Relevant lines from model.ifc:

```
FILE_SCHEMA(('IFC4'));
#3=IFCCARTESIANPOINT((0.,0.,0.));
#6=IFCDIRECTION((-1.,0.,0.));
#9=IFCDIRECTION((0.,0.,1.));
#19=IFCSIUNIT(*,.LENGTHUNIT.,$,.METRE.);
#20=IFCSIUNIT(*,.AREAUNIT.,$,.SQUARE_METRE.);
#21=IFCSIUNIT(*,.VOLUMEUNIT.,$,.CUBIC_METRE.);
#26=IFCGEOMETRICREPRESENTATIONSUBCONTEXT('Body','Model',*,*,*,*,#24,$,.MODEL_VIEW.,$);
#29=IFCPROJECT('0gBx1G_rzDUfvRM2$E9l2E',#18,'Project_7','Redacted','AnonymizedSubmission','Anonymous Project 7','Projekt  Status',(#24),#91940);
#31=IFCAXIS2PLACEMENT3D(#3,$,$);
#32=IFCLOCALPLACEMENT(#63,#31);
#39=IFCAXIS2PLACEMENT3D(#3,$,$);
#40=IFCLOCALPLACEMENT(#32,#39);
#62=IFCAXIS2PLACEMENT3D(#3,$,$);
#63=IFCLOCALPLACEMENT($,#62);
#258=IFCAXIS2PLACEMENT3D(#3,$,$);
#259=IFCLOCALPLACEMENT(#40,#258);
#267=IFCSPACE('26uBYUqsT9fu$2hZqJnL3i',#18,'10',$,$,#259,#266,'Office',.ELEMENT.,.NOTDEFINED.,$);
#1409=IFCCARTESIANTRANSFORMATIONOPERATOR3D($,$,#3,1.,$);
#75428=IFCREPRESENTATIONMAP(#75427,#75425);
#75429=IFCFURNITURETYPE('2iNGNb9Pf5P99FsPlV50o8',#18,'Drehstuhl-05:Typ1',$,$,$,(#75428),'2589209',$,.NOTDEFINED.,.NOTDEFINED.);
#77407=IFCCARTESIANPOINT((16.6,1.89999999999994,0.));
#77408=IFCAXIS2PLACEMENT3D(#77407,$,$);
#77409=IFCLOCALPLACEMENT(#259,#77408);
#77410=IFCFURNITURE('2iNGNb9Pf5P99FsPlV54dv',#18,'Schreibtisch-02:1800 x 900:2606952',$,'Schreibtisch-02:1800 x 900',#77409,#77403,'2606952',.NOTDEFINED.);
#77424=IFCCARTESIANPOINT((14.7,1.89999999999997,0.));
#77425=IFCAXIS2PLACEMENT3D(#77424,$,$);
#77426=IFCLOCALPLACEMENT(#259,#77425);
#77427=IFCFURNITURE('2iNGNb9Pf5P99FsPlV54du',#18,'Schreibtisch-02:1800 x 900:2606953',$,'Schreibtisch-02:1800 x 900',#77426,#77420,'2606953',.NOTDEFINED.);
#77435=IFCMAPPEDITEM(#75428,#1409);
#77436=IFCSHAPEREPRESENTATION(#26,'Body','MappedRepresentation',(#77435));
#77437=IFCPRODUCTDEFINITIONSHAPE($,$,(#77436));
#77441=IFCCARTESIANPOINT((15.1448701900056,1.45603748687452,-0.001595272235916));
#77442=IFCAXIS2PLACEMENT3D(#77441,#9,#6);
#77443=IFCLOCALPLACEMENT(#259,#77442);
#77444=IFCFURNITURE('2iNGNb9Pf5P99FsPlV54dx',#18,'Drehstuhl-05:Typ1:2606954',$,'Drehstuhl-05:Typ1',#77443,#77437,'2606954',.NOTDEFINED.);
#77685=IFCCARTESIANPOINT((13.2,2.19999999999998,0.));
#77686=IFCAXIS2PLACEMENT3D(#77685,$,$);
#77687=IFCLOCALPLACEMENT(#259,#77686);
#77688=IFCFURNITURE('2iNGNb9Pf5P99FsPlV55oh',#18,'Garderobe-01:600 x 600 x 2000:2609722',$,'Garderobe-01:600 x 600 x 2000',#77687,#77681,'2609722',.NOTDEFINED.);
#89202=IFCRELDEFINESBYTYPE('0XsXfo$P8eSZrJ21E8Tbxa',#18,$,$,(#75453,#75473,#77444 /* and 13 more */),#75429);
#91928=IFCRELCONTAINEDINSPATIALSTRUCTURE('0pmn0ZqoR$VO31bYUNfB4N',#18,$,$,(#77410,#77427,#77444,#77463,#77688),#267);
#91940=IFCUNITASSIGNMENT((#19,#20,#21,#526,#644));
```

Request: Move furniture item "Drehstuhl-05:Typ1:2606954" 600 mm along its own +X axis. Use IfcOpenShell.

```python
import ifcopenshell
import ifcopenshell.api.geometry
import ifcopenshell.util.placement

model = ifcopenshell.open("model.ifc")

item = model.by_id(77444)
matrix = ifcopenshell.util.placement.get_local_placement(item.ObjectPlacement)
matrix[:3, 3] += matrix[:3, 0] * 0.6
ifcopenshell.api.geometry.edit_object_placement(model, product=item, matrix=matrix, is_si=False)

print(ifcopenshell.util.placement.get_local_placement(item.ObjectPlacement).round(3) + 0.0)

model.write("model_rev.ifc")
```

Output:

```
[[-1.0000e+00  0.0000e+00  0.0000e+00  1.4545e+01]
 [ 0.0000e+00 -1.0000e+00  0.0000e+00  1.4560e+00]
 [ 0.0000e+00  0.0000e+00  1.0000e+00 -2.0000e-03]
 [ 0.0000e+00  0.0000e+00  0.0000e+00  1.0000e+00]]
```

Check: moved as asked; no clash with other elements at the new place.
